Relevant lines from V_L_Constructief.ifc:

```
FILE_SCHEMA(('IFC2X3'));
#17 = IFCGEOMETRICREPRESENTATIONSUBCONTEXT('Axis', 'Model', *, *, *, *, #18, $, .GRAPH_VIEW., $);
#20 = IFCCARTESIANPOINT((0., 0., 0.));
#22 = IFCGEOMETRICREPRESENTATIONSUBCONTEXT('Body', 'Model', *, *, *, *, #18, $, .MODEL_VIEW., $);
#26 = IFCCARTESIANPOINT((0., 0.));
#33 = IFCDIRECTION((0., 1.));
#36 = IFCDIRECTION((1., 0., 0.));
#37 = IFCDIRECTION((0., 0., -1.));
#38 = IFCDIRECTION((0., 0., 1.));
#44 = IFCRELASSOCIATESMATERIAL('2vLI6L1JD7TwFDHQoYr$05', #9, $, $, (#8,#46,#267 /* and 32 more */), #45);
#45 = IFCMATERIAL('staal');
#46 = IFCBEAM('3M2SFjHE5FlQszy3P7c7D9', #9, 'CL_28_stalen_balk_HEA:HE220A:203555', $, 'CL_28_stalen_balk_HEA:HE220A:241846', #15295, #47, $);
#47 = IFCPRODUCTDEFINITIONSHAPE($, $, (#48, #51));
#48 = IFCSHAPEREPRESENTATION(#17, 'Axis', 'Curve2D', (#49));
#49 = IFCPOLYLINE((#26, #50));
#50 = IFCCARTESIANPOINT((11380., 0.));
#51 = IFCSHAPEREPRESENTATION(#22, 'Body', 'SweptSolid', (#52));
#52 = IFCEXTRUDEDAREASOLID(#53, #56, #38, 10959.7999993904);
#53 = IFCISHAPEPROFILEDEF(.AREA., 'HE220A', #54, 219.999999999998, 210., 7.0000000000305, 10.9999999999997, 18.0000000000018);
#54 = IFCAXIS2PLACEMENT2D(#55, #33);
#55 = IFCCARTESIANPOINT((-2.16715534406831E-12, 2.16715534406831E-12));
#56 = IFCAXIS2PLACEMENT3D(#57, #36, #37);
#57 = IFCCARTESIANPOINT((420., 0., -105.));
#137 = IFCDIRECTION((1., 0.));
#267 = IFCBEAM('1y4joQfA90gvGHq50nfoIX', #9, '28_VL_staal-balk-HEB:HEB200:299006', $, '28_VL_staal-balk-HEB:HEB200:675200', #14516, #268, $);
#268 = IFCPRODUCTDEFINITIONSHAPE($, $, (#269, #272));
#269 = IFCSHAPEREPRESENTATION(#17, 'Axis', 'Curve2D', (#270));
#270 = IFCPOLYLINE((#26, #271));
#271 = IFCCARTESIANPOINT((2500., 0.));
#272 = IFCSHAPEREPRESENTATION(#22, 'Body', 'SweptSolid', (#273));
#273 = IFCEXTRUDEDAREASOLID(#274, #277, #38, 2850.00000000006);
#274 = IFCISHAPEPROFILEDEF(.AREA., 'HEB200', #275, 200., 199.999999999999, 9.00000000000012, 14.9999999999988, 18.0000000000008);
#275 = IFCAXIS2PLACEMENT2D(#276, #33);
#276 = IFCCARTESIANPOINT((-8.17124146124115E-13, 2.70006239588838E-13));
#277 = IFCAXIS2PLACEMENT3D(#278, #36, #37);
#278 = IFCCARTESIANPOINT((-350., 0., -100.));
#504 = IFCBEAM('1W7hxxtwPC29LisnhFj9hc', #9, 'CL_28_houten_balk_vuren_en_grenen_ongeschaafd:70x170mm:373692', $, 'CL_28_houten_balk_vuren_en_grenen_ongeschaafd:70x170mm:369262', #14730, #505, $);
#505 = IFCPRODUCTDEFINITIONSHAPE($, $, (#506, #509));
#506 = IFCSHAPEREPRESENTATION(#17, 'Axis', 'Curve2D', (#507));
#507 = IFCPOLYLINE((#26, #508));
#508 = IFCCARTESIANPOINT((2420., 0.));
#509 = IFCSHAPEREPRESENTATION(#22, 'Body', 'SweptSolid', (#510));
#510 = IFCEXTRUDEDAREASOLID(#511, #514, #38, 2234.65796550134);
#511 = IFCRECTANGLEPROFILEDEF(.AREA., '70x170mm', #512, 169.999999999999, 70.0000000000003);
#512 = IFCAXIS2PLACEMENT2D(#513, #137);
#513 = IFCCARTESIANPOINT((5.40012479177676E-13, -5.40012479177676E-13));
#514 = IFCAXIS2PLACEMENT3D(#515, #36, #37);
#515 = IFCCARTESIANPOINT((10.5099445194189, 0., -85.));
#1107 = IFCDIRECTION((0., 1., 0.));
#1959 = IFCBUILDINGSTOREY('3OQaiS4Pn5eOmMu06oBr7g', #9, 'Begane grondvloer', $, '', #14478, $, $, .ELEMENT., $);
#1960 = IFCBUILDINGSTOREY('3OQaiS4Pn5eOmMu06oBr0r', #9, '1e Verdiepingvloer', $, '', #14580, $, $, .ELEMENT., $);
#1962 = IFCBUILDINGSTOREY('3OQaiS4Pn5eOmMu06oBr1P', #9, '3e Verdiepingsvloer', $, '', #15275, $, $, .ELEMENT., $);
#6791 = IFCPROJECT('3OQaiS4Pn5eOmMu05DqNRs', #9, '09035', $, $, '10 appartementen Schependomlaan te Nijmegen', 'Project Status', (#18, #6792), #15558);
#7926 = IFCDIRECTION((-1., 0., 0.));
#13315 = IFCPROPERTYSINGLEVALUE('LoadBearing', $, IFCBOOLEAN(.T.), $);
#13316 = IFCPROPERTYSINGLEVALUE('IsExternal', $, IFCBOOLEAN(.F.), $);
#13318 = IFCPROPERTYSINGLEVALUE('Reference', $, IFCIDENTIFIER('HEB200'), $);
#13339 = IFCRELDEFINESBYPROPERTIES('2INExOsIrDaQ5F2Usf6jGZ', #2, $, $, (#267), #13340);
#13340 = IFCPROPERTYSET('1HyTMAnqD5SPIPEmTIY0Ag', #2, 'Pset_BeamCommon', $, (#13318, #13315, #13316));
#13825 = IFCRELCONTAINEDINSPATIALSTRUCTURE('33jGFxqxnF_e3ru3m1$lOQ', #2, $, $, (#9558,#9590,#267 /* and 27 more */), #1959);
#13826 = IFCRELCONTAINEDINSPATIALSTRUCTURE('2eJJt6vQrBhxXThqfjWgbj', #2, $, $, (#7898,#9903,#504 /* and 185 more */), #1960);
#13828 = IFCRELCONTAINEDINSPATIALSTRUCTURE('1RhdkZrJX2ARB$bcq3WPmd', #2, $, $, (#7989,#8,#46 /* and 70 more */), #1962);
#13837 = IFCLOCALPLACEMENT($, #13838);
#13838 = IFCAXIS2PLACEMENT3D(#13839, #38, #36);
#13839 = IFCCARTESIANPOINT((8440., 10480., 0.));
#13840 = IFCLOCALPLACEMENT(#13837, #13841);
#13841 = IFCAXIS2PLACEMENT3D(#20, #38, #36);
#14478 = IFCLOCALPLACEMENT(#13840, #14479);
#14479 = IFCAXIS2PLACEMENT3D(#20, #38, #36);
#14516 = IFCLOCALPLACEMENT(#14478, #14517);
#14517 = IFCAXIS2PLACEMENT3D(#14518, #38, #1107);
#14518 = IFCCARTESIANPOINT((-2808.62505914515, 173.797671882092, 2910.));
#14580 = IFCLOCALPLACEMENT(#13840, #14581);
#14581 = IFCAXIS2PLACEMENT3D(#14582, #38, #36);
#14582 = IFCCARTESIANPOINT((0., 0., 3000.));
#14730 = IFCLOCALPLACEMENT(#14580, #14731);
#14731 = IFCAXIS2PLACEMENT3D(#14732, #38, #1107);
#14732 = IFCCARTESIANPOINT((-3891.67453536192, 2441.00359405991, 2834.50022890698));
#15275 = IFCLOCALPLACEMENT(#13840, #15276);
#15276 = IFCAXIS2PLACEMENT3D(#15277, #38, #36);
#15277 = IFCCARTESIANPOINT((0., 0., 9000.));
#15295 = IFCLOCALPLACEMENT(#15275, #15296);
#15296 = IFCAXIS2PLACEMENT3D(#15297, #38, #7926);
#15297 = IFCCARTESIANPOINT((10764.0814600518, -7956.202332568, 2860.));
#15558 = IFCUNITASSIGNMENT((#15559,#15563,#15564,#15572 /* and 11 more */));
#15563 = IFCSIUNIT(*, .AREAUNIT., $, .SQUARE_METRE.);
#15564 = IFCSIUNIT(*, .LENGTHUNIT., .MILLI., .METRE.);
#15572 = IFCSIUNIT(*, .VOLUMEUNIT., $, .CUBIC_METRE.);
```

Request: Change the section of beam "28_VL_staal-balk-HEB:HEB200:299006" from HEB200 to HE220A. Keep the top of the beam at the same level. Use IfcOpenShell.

```python
import ifcopenshell
import ifcopenshell.api.pset
import ifcopenshell.util.element
import ifcopenshell.util.representation

model = ifcopenshell.open("V_L_Constructief.ifc")

member = model.by_guid("1y4joQfA90gvGHq50nfoIX")
source = next(p for p in model.by_type("IfcIShapeProfileDef") if p.ProfileName == "HE220A")

body = ifcopenshell.util.representation.get_representation(member, "Model", "Body")
solid = body.Items[0]
old_profile = solid.SweptArea

# Copy the section's sizes but keep this member's own profile position.
profile = ifcopenshell.util.element.copy(model, source)
# Profiles are centred, so shift by half the change in depth to hold the top.
shift = (old_profile.OverallDepth - profile.OverallDepth) / 2
x, y = old_profile.Position.Location.Coordinates
up = (-1.0, 0.0)  # upwards, in the solid's own plane
location = model.createIfcCartesianPoint((x + up[0] * shift, y + up[1] * shift))
profile.Position = model.createIfcAxis2Placement2D(location, old_profile.Position.RefDirection)
solid.SweptArea = profile
if not model.get_total_inverses(old_profile):
    ifcopenshell.util.element.remove_deep2(model, old_profile)
member.Name = member.Name.replace("HEB200", "HE220A")
member.ObjectType = member.ObjectType.replace("HEB200", "HE220A")
pset = model.by_id(ifcopenshell.util.element.get_pset(member, "Pset_BeamCommon", should_inherit=False)["id"])
ifcopenshell.api.pset.edit_pset(model, pset=pset, properties={"Reference": "HE220A"})

print(solid.SweptArea)

model.write("V_L_Constructief_v2.ifc")
```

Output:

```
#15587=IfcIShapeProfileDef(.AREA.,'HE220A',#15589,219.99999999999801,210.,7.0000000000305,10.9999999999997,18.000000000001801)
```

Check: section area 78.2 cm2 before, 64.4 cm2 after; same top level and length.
